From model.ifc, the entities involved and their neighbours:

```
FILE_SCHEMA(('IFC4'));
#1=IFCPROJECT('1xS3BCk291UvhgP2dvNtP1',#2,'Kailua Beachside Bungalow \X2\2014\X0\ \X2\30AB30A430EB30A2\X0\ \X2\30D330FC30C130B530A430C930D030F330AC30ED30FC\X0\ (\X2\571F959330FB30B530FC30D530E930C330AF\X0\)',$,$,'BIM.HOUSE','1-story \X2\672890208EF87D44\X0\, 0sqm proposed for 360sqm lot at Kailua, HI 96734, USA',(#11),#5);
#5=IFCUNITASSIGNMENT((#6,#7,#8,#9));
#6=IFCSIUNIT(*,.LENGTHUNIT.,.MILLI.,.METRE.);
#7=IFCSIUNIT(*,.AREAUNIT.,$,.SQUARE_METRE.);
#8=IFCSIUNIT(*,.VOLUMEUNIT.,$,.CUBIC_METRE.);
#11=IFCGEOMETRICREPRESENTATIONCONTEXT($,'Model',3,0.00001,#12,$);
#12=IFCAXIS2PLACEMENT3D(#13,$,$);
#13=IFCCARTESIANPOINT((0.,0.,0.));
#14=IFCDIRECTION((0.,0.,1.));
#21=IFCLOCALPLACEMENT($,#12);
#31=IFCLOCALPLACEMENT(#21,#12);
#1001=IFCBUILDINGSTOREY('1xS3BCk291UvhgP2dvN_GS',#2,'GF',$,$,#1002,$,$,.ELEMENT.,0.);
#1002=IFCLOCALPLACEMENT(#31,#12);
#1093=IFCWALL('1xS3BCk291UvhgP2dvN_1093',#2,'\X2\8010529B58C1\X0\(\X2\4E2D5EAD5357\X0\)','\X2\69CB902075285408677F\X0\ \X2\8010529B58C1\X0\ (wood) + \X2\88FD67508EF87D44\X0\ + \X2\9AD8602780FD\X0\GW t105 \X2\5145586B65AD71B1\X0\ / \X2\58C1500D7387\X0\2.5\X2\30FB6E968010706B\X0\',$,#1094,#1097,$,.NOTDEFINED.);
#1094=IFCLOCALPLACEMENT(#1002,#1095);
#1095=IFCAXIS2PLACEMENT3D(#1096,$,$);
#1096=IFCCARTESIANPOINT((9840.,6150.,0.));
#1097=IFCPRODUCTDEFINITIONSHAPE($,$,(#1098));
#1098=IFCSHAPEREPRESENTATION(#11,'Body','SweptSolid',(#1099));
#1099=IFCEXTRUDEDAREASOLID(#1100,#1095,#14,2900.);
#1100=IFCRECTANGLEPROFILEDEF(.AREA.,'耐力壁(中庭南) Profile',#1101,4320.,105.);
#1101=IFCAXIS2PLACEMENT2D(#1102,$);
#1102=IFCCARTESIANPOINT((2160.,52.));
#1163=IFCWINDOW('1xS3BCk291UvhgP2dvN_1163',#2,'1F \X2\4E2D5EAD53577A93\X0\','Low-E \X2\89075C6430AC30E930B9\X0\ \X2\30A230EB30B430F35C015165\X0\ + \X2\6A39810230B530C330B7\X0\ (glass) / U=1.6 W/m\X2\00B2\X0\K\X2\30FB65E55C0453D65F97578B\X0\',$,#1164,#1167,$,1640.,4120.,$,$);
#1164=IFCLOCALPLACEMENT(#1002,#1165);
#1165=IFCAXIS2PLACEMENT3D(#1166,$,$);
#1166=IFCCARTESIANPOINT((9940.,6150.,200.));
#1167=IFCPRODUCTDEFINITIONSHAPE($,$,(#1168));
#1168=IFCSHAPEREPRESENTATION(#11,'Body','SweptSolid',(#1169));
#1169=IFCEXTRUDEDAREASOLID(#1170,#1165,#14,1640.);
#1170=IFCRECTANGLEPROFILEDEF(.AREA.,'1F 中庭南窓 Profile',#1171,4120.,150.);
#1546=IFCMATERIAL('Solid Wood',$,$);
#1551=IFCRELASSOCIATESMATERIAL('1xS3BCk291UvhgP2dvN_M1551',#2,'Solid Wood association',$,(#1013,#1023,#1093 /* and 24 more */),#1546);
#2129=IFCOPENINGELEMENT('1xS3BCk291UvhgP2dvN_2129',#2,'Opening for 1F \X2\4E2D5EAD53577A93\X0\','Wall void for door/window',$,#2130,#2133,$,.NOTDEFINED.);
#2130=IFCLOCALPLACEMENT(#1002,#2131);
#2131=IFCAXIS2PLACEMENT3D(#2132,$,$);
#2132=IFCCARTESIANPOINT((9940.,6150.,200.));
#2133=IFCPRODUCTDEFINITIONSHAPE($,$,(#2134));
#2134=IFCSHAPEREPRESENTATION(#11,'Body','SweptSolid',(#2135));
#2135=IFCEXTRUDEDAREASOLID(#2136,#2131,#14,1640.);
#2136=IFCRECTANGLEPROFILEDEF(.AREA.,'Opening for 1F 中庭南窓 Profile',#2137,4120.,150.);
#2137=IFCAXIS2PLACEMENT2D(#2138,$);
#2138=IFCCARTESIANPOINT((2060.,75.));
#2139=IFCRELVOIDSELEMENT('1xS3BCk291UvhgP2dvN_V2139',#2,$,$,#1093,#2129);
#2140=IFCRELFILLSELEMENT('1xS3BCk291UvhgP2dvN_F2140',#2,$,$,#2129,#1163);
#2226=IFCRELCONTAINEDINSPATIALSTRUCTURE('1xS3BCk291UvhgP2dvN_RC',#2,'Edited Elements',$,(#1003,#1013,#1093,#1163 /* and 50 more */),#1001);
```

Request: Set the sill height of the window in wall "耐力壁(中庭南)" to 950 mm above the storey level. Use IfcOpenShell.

```python
import numpy as np
import ifcopenshell
import ifcopenshell.api.geometry
import ifcopenshell.geom
import ifcopenshell.util.element
import ifcopenshell.util.placement
import ifcopenshell.util.shape
import ifcopenshell.util.unit

model = ifcopenshell.open("model.ifc")
unit_scale = ifcopenshell.util.unit.calculate_unit_scale(model)

window = model.by_guid("1xS3BCk291UvhgP2dvN_1163")
opening = window.FillsVoids[0].RelatingOpeningElement
storey = ifcopenshell.util.element.get_container(window, ifc_class="IfcBuildingStorey")
level = ifcopenshell.util.placement.get_local_placement(storey.ObjectPlacement)[2, 3]

# The opening's origin need not be at the sill, so measure its lowest point.
shape = ifcopenshell.geom.create_shape(ifcopenshell.geom.settings(), opening)
bottom = ifcopenshell.util.shape.get_shape_bottom_elevation(shape, shape.geometry) / unit_scale
dz = level + 0.95 / unit_scale - bottom

shift = np.array([0.0, 0.0, dz])
# The window is not placed relative to its opening, so move both.
for product in (opening, window):
    matrix = ifcopenshell.util.placement.get_local_placement(product.ObjectPlacement)
    matrix[:3, 3] += shift
    ifcopenshell.api.geometry.edit_object_placement(model, product=product, matrix=matrix, is_si=False)

print(f"moved by {dz * unit_scale:+.3f} m")

model.write("model_updated.ifc")
```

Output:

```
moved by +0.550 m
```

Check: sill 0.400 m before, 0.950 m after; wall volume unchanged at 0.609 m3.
